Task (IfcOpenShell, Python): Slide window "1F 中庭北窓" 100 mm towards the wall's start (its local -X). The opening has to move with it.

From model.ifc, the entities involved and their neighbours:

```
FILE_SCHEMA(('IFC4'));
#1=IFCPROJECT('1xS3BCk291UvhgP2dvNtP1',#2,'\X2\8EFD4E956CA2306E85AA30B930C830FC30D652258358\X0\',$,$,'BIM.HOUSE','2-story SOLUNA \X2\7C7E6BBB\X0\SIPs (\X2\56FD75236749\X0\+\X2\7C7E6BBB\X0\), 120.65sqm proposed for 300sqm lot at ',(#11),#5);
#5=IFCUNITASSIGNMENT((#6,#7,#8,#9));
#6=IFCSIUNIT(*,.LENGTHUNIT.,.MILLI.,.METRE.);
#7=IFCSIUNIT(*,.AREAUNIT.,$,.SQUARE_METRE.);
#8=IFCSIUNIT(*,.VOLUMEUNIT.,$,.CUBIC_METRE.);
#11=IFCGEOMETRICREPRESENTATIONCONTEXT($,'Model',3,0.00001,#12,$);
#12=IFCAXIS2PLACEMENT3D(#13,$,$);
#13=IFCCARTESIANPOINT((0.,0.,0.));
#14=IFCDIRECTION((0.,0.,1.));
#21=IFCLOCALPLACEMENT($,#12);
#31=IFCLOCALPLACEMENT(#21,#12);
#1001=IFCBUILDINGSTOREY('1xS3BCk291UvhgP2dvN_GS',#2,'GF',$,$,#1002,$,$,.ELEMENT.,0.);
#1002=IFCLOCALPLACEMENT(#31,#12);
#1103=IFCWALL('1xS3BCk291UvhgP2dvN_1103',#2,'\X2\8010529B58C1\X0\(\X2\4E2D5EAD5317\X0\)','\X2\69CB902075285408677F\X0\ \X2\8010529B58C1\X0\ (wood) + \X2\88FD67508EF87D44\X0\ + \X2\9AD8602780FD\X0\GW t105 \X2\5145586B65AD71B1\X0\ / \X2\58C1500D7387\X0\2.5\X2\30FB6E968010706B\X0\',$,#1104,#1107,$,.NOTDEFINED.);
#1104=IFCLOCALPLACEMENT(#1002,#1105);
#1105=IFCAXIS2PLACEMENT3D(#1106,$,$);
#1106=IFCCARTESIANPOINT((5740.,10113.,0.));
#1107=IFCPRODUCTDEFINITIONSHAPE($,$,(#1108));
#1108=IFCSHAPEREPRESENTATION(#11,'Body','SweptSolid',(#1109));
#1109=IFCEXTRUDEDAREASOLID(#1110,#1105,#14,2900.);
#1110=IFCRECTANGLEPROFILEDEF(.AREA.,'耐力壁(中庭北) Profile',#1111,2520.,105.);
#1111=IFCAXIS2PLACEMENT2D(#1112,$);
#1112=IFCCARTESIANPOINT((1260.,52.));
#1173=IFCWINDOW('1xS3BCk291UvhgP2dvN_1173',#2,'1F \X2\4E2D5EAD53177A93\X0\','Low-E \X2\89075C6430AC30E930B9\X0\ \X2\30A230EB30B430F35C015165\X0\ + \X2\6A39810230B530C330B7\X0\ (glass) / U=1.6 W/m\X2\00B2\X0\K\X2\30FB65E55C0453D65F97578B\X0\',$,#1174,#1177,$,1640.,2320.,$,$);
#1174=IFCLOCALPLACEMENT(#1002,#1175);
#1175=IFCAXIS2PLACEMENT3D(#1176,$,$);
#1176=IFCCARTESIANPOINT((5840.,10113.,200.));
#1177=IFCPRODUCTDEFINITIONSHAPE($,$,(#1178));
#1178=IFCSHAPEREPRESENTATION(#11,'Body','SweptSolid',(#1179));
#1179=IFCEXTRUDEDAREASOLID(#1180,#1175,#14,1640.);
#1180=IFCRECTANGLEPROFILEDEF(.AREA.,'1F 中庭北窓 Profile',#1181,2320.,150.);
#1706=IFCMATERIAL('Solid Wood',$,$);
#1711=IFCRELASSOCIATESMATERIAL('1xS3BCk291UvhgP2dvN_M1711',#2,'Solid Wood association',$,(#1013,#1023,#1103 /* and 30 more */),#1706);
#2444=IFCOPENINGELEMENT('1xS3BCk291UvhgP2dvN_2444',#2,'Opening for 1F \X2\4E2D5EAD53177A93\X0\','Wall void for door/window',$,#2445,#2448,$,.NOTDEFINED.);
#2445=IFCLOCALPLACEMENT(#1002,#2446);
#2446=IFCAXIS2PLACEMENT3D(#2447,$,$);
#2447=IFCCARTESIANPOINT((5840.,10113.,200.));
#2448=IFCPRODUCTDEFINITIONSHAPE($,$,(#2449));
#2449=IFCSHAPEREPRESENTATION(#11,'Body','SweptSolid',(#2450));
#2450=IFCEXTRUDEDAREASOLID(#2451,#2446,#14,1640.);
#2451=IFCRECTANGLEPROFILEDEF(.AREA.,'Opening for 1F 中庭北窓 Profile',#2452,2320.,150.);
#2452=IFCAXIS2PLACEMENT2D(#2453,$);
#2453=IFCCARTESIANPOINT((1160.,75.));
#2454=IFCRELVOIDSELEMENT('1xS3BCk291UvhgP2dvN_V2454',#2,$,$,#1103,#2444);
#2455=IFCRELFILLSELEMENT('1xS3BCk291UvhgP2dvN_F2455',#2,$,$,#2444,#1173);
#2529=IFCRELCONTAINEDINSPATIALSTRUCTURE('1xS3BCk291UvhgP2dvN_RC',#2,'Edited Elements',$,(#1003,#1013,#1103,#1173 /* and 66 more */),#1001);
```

```python
import ifcopenshell
import ifcopenshell.api.geometry
import ifcopenshell.util.placement

model = ifcopenshell.open("model.ifc")

window = model.by_guid("1xS3BCk291UvhgP2dvN_1173")
opening = window.FillsVoids[0].RelatingOpeningElement
wall = opening.VoidsElements[0].RelatingBuildingElement

wall_matrix = ifcopenshell.util.placement.get_local_placement(wall.ObjectPlacement)
shift = wall_matrix[:3, 0] * -100.0
before = ifcopenshell.util.placement.get_local_placement(window.ObjectPlacement)[:3, 3].copy()

# The window is not placed relative to its opening, so move both.
for product in (opening, window):
    matrix = ifcopenshell.util.placement.get_local_placement(product.ObjectPlacement)
    matrix[:3, 3] += shift
    ifcopenshell.api.geometry.edit_object_placement(model, product=product, matrix=matrix, is_si=False)

after = ifcopenshell.util.placement.get_local_placement(window.ObjectPlacement)[:3, 3]
print("window moved by", (after - before).round(3) + 0.0)

model.write("model_edited.ifc")
```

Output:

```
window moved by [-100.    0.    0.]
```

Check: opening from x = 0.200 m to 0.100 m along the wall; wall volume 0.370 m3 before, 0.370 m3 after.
